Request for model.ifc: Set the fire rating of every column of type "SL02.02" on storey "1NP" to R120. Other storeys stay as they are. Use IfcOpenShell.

First a look at what the model holds.

```python
import ifcopenshell
import ifcopenshell.util.element

model = ifcopenshell.open("model.ifc")
print(model.schema)
storey = next(s for s in model.by_type("IfcBuildingStorey") if s.Name == "1NP")
columns = [e for e in ifcopenshell.util.element.get_decomposition(storey) if e.is_a("IfcColumn")]
seen = {}
for e in columns:
    element_type = ifcopenshell.util.element.get_type(e)
    key = (element_type.Name if element_type != e and element_type else None, ifcopenshell.util.element.get_pset(e, "Pset_ColumnCommon", "FireRating"))
    seen[key] = seen.get(key, 0) + 1
for (name, value), count in sorted(seen.items(), key=str):
    print(count, "x", name, "|", value)
```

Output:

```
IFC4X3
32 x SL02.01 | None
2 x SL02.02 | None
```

```python
import ifcopenshell
import ifcopenshell.api.pset
import ifcopenshell.util.element

model = ifcopenshell.open("model.ifc")

storey = next(s for s in model.by_type("IfcBuildingStorey") if s.Name == "1NP")
columns = [e for e in ifcopenshell.util.element.get_decomposition(storey) if e.is_a("IfcColumn")]

count = 0
for e in columns:
    element_type = ifcopenshell.util.element.get_type(e)
    if element_type in (None, e) or element_type.Name != "SL02.02":
        continue
    # add_pset returns the element's existing set when there is one.
    pset = ifcopenshell.api.pset.add_pset(model, product=e, name="Pset_ColumnCommon")
    ifcopenshell.api.pset.edit_pset(model, pset=pset, properties={"FireRating": "R120"})
    count += 1

print(count, "columns updated")

model.write("model-out.ifc")
```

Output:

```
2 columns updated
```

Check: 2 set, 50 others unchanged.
